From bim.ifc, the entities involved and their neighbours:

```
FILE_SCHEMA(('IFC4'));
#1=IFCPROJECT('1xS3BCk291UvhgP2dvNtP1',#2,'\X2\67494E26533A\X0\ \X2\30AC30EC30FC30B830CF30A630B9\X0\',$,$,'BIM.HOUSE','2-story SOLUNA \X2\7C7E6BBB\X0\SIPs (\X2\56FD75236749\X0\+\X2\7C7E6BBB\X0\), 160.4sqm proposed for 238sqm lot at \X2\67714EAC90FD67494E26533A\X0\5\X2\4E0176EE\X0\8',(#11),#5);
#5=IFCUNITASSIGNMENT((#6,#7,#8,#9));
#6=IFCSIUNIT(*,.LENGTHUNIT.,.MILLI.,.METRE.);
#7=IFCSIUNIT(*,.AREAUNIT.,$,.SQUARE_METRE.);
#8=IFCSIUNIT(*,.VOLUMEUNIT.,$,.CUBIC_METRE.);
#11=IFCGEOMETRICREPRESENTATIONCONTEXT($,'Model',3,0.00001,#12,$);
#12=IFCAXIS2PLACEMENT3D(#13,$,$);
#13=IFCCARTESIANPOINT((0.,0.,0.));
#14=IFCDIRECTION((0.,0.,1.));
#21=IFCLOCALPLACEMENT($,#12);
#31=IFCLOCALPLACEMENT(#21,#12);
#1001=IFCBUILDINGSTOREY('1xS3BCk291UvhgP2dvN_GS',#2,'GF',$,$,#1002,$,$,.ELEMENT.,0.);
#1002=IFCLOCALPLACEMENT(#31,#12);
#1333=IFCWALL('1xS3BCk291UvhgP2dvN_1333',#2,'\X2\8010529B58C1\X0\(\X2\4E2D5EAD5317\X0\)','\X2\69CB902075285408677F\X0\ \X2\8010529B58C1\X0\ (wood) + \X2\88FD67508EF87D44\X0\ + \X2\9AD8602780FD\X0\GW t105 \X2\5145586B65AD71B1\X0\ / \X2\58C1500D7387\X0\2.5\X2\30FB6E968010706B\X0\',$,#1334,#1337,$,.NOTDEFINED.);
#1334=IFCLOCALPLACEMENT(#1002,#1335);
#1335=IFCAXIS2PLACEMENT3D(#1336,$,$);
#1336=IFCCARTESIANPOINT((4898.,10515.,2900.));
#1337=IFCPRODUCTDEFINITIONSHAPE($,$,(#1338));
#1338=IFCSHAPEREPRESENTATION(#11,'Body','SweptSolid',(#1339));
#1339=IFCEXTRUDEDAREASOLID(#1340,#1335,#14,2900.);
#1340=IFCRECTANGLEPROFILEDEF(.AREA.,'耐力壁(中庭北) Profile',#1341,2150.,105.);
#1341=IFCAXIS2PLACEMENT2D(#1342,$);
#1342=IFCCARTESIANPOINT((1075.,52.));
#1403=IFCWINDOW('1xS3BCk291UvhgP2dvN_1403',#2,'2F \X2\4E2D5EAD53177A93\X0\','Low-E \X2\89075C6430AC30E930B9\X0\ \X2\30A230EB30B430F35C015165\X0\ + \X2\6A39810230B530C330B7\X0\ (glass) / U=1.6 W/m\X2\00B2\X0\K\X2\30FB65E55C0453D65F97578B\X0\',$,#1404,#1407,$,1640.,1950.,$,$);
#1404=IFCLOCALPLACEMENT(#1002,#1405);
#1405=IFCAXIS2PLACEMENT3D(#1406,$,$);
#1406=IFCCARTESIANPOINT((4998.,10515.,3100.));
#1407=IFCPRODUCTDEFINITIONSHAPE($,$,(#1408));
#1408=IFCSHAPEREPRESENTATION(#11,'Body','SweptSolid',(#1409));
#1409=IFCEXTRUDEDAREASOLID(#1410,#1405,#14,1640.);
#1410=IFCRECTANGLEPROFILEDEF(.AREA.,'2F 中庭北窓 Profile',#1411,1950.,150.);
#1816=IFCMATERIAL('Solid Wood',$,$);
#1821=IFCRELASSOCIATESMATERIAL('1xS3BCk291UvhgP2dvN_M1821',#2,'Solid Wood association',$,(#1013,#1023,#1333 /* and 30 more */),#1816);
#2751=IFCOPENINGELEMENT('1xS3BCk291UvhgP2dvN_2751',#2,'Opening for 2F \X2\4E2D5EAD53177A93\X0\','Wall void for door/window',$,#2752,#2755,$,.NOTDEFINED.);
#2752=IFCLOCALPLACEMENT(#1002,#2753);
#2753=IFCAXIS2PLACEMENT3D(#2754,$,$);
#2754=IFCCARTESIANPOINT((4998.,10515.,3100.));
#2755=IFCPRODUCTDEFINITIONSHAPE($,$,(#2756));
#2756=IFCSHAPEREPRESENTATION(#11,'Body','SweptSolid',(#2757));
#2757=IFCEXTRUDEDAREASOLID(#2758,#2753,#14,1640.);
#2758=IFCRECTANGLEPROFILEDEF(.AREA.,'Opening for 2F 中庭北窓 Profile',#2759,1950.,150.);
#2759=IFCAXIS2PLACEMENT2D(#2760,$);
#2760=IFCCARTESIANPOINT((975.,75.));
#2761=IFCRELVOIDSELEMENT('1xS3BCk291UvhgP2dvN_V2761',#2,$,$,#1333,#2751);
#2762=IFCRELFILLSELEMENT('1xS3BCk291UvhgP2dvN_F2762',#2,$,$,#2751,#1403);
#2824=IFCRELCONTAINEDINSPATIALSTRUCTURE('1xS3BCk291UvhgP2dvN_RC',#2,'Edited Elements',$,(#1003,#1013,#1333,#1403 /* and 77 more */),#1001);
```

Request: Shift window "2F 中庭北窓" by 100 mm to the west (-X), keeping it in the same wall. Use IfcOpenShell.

```python
import ifcopenshell
import ifcopenshell.api.geometry
import ifcopenshell.util.placement
import ifcopenshell.util.unit

model = ifcopenshell.open("bim.ifc")
unit_scale = ifcopenshell.util.unit.calculate_unit_scale(model)

window = model.by_guid("1xS3BCk291UvhgP2dvN_1403")
opening = window.FillsVoids[0].RelatingOpeningElement
wall = opening.VoidsElements[0].RelatingBuildingElement

wall_matrix = ifcopenshell.util.placement.get_local_placement(wall.ObjectPlacement)
shift = wall_matrix[:3, 0] * -0.1 / unit_scale
before = ifcopenshell.util.placement.get_local_placement(window.ObjectPlacement)[:3, 3].copy()

# The window is not placed relative to its opening, so move both.
for product in (opening, window):
    matrix = ifcopenshell.util.placement.get_local_placement(product.ObjectPlacement)
    matrix[:3, 3] += shift
    ifcopenshell.api.geometry.edit_object_placement(model, product=product, matrix=matrix, is_si=False)

after = ifcopenshell.util.placement.get_local_placement(window.ObjectPlacement)[:3, 3]
print("window moved by", (after - before).round(3) + 0.0)

model.write("bim-out.ifc")
```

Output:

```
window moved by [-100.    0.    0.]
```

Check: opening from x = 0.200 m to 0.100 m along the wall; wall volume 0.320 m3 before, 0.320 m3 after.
